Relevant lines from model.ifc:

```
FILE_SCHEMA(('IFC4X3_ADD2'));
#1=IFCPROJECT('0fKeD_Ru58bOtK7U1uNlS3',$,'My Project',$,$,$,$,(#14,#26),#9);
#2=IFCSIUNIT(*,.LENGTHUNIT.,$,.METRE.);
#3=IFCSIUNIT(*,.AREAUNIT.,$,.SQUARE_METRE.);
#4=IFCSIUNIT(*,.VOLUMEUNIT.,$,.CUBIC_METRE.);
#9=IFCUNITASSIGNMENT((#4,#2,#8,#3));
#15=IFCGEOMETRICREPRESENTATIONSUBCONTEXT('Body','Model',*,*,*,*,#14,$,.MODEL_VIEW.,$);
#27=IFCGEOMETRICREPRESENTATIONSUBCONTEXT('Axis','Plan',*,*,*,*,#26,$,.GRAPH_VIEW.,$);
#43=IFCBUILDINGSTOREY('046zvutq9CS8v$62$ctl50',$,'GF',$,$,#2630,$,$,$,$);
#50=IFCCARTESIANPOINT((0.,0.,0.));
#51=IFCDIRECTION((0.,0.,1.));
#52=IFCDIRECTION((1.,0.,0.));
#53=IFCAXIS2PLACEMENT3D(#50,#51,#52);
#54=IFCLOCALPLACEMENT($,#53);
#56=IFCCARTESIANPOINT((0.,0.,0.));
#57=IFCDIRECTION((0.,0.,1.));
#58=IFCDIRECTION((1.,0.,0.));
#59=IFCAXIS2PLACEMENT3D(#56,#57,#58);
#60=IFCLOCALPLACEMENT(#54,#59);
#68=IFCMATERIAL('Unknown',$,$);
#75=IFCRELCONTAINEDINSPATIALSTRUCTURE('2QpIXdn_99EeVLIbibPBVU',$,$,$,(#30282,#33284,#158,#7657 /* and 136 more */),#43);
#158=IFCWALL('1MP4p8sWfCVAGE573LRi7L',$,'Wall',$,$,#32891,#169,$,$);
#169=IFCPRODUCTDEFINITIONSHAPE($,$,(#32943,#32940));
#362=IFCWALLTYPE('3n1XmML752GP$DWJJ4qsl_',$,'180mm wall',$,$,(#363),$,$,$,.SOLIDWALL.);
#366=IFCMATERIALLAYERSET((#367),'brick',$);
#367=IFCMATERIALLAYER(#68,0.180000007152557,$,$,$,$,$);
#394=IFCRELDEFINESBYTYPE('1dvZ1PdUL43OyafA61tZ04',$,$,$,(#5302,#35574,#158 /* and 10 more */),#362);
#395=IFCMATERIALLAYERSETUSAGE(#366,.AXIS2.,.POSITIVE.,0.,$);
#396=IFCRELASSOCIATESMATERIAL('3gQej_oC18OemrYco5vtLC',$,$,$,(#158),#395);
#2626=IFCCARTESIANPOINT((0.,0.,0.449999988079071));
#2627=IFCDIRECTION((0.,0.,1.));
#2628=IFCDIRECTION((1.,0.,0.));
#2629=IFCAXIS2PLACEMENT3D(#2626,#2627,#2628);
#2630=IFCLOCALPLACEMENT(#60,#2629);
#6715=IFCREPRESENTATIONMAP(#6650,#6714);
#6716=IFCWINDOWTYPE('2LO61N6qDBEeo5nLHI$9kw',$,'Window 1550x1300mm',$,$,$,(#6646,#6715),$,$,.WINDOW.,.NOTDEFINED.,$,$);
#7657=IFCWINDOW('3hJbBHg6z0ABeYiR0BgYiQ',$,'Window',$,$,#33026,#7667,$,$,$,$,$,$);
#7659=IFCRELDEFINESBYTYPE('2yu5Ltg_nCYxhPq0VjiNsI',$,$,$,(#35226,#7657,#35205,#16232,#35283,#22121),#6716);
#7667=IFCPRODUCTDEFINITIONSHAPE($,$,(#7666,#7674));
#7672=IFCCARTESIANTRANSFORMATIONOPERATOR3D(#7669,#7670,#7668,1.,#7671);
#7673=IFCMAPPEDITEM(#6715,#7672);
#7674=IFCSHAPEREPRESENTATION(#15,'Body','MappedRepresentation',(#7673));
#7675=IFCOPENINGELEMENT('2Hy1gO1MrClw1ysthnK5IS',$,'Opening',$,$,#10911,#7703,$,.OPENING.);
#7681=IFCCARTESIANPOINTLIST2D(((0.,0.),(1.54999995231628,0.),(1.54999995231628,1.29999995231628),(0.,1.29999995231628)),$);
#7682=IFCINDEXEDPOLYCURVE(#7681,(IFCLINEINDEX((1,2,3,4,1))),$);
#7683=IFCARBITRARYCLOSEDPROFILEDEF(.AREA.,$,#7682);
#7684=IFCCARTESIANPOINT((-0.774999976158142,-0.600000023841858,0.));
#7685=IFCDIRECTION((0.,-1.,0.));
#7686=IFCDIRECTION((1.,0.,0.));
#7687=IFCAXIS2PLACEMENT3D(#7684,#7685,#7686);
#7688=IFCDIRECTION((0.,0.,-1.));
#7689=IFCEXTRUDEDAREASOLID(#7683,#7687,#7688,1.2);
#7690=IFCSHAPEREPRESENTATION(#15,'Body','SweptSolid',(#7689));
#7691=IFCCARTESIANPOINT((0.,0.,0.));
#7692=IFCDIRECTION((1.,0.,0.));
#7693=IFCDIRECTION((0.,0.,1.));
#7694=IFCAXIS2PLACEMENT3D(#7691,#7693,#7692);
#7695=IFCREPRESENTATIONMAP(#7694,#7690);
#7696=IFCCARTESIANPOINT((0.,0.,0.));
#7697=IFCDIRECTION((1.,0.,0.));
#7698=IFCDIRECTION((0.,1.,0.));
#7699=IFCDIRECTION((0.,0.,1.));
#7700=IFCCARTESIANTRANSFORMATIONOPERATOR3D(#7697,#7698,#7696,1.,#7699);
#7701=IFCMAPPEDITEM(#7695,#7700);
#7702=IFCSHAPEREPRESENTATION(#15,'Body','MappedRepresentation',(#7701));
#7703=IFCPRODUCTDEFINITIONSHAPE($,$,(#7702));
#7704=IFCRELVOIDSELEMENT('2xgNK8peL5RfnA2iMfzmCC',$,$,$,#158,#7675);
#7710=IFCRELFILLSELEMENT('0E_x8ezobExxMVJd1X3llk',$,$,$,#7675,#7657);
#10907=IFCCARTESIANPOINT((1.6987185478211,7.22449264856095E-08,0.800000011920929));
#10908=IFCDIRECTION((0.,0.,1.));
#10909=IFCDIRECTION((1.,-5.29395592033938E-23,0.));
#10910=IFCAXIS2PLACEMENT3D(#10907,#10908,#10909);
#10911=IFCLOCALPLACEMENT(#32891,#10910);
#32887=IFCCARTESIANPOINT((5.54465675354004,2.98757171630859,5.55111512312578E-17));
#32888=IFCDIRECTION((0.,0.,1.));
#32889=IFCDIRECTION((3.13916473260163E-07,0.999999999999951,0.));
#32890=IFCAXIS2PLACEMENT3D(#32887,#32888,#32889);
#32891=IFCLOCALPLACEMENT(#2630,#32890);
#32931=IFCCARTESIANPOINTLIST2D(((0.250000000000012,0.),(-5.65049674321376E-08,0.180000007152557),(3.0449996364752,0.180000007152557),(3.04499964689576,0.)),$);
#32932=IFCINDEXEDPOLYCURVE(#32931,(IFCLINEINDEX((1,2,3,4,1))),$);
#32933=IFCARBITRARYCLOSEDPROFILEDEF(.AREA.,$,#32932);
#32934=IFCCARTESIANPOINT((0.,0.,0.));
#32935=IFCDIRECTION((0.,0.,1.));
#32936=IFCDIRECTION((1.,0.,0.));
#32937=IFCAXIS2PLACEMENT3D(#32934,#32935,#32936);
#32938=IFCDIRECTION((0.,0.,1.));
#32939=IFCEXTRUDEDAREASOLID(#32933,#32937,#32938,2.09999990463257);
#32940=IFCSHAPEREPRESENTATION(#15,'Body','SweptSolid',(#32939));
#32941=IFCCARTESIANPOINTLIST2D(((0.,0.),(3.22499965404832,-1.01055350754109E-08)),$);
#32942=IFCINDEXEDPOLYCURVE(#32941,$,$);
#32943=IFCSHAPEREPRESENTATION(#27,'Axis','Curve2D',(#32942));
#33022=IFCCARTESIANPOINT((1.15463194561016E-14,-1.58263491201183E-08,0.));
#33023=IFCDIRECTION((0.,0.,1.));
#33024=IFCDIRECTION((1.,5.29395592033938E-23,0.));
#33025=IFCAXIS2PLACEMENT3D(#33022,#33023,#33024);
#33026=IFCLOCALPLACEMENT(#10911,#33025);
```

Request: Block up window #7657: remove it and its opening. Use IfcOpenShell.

```python
import ifcopenshell
import ifcopenshell.api.feature
import ifcopenshell.api.root
import ifcopenshell.geom
import ifcopenshell.util.shape

model = ifcopenshell.open("model.ifc")
settings = ifcopenshell.geom.settings()


def volume(element):
    """Net volume in cubic metres, openings subtracted."""
    shape = ifcopenshell.geom.create_shape(settings, element)
    return ifcopenshell.util.shape.get_volume(shape.geometry)


window = model.by_guid("3hJbBHg6z0ABeYiR0BgYiQ")
opening = window.FillsVoids[0].RelatingOpeningElement
wall = opening.VoidsElements[0].RelatingBuildingElement
before = volume(wall)

ifcopenshell.api.root.remove_product(model, product=window)
ifcopenshell.api.feature.remove_feature(model, feature=opening)

after = volume(wall)

print(f"wall volume {before:.3f} -> {after:.3f} m3")

model.write("model-out.ifc")
```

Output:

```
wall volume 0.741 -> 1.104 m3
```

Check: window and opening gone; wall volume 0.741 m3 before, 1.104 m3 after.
